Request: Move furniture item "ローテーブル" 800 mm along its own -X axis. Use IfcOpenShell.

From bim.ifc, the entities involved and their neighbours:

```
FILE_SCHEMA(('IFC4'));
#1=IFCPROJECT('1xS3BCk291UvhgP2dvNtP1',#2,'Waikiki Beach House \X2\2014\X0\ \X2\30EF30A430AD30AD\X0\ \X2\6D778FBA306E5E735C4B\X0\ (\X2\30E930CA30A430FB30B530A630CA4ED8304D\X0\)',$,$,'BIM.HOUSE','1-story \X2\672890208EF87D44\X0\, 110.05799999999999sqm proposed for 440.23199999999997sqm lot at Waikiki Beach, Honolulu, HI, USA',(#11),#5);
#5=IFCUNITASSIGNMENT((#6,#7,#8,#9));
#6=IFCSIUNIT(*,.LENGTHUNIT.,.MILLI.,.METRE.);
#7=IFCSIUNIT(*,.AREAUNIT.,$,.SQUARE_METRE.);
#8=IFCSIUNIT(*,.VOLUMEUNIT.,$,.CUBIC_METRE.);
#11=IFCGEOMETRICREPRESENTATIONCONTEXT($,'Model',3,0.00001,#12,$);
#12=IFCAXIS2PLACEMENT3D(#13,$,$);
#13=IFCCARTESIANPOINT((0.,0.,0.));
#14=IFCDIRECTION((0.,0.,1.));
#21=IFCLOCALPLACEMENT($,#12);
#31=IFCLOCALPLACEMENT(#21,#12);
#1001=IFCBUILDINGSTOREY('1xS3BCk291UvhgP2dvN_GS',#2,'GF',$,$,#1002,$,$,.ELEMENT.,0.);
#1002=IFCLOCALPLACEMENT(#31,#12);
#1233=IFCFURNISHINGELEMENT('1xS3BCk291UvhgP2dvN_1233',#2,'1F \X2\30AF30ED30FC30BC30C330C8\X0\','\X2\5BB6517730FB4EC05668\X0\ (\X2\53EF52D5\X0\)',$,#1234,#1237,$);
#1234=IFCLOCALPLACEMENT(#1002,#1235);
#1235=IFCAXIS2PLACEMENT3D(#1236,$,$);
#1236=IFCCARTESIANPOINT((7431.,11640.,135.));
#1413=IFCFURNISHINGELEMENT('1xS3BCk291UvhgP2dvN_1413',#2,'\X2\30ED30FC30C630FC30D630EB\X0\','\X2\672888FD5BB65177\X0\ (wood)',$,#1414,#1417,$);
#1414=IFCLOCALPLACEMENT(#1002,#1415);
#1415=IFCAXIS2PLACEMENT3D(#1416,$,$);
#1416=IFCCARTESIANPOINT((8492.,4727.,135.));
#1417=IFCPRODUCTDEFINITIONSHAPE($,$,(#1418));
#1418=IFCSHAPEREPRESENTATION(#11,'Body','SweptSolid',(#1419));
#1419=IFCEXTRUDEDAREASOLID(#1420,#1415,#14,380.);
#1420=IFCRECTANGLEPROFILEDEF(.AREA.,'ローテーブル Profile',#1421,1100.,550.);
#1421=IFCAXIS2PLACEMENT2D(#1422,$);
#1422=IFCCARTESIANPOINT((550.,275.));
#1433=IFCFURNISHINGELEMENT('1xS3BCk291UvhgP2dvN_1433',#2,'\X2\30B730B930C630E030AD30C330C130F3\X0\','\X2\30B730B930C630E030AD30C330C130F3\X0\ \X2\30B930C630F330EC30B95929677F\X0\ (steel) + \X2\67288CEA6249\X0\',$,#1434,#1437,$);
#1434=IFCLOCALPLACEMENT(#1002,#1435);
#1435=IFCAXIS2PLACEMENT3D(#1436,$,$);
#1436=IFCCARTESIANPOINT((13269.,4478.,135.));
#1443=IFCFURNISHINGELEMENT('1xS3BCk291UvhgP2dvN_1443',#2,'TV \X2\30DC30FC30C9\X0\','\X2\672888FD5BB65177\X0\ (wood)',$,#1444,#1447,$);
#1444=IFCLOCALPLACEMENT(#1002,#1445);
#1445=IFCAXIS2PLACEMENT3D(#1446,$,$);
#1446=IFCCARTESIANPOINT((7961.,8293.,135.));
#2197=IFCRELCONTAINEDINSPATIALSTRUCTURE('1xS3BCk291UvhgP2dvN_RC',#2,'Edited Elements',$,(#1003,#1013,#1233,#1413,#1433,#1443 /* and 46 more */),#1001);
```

```python
import ifcopenshell
import ifcopenshell.api.geometry
import ifcopenshell.util.placement

model = ifcopenshell.open("bim.ifc")

item = model.by_guid("1xS3BCk291UvhgP2dvN_1413")
matrix = ifcopenshell.util.placement.get_local_placement(item.ObjectPlacement)
matrix[:3, 3] -= matrix[:3, 0] * 800.0
ifcopenshell.api.geometry.edit_object_placement(model, product=item, matrix=matrix, is_si=False)

print(ifcopenshell.util.placement.get_local_placement(item.ObjectPlacement).round(3) + 0.0)

model.write("bim_edited.ifc")
```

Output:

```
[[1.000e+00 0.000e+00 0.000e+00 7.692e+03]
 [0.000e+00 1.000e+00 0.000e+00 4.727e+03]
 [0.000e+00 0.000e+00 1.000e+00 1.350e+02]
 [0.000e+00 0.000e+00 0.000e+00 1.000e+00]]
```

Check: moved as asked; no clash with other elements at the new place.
